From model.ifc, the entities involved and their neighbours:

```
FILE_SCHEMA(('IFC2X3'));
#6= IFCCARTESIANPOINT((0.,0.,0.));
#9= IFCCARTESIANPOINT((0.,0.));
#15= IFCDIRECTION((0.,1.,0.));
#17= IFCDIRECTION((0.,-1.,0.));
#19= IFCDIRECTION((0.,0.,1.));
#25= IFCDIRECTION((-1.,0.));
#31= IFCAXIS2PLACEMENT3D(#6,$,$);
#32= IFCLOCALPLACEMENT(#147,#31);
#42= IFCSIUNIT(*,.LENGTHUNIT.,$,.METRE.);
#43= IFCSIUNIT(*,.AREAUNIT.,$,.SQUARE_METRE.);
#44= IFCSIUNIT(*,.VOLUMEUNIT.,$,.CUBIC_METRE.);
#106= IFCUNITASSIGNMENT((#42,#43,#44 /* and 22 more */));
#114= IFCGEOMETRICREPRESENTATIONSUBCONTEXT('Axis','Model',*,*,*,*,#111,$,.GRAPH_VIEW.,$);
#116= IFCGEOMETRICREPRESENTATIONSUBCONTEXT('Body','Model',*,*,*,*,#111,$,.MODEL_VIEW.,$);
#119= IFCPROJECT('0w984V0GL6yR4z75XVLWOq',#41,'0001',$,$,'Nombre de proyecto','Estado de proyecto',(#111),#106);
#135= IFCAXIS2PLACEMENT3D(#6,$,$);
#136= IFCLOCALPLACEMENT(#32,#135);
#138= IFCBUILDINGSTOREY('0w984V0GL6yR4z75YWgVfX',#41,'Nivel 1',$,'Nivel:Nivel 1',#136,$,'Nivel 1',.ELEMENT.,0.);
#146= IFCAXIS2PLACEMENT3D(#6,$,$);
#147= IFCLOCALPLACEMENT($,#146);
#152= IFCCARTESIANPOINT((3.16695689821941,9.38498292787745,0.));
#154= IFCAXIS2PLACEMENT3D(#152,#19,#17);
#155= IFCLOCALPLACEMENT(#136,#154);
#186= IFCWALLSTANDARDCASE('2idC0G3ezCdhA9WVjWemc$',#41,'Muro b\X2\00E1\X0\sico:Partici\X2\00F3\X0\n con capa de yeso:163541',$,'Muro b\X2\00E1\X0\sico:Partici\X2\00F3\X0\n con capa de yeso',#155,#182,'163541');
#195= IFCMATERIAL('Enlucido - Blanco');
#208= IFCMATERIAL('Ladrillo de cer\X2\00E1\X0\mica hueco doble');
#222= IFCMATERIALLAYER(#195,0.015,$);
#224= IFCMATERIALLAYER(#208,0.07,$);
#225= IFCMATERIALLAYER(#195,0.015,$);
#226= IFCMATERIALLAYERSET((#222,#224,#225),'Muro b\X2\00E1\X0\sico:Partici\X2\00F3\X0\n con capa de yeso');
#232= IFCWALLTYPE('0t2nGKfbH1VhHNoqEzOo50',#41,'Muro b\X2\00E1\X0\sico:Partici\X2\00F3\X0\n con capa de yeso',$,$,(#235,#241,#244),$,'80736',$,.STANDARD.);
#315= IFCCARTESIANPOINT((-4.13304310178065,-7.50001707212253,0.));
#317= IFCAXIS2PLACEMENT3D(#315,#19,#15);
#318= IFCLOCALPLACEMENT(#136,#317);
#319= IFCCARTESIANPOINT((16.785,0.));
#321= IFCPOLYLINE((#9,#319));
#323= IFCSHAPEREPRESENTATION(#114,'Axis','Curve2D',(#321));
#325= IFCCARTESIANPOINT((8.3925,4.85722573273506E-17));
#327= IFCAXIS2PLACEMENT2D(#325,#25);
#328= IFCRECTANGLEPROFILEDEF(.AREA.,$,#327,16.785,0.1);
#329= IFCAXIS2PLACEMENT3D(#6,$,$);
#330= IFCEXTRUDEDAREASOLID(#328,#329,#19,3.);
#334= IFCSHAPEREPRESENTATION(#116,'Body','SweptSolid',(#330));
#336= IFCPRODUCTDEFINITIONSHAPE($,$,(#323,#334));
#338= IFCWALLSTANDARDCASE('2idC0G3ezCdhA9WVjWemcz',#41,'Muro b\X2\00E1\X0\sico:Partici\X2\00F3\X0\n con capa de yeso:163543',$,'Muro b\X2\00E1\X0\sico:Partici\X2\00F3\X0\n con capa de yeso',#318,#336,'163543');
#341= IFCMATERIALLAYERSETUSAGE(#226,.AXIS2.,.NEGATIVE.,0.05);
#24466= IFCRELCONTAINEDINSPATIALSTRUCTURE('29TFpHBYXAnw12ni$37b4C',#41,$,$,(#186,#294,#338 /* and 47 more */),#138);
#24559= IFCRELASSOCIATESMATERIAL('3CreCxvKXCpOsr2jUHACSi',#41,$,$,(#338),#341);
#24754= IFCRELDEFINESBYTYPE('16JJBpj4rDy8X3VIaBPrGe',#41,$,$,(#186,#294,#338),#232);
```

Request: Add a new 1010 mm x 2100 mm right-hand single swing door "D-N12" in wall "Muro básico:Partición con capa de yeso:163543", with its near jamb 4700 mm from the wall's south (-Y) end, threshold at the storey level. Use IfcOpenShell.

```python
import numpy as np
import ifcopenshell
import ifcopenshell.api.feature
import ifcopenshell.api.geometry
import ifcopenshell.api.root
import ifcopenshell.api.spatial
import ifcopenshell.api.type
import ifcopenshell.geom
import ifcopenshell.util.element
import ifcopenshell.util.placement
import ifcopenshell.util.representation
import ifcopenshell.util.shape
import ifcopenshell.util.unit

model = ifcopenshell.open("model.ifc")
unit_scale = ifcopenshell.util.unit.calculate_unit_scale(model)
settings = ifcopenshell.geom.settings()


def volume(element):
    """Net volume in cubic metres, openings subtracted."""
    shape = ifcopenshell.geom.create_shape(settings, element)
    return ifcopenshell.util.shape.get_volume(shape.geometry)


wall = model.by_id(338)
storey = ifcopenshell.util.element.get_container(wall, ifc_class="IfcBuildingStorey")
context = ifcopenshell.util.representation.get_context(model, "Model", "Body", "MODEL_VIEW")
before = volume(wall)

width, height, from_end, sill = 1.01, 2.1, 4.7, 0.0  # metres

# The wall runs along its own X axis, and the end named is its -X end.
wall_shape = ifcopenshell.geom.create_shape(settings, wall)
x, y, z = ifcopenshell.util.shape.get_vertices(wall_shape.geometry).T
start = x.min() + from_end
face, thickness = float(y.min()), float(y.max() - y.min())
wall_matrix = ifcopenshell.util.placement.get_local_placement(wall.ObjectPlacement)
level = ifcopenshell.util.placement.get_local_placement(storey.ObjectPlacement)[2, 3]


def in_wall(x, y):
    """Placement at x, y metres in the wall's axes, at sill height."""
    matrix = wall_matrix.copy()
    matrix[:, 3] = wall_matrix @ np.array([x / unit_scale, y / unit_scale, 0.0, 1.0])
    matrix[2, 3] = level + sill / unit_scale
    return matrix


# Opening: a box that overshoots both wall faces by 50 mm.
opening = ifcopenshell.api.root.create_entity(model, ifc_class="IfcOpeningElement")
box = ifcopenshell.api.geometry.add_wall_representation(
    model, context=context, length=width, height=height, thickness=thickness + 0.1
)
ifcopenshell.api.geometry.assign_representation(model, product=opening, representation=box)
ifcopenshell.api.geometry.edit_object_placement(model, product=opening, matrix=in_wall(start, face - 0.05), is_si=False)
ifcopenshell.api.feature.add_feature(model, feature=opening, element=wall)

door = ifcopenshell.api.root.create_entity(model, ifc_class="IfcDoor", name="D-N12")
door.OverallWidth, door.OverallHeight = width / unit_scale, height / unit_scale
body = ifcopenshell.api.geometry.add_door_representation(
    model,
    context=context,
    overall_width=door.OverallWidth,
    overall_height=door.OverallHeight,
    operation_type="SINGLE_SWING_RIGHT",
    lining_properties={"LiningDepth": thickness / unit_scale, "ThresholdDepth": thickness / unit_scale},
)
ifcopenshell.api.geometry.assign_representation(model, product=door, representation=body)
ifcopenshell.api.spatial.assign_container(model, products=[door], relating_structure=storey)
fills = ifcopenshell.api.feature.add_filling(model, opening=opening, element=door)
fills.OwnerHistory = door.OwnerHistory  # required in IFC2X3

# IFC2X3 keeps the operation on the door style.
style = ifcopenshell.api.root.create_entity(model, ifc_class="IfcDoorStyle", name="D-N12")
style.OperationType, style.ConstructionType = "SINGLE_SWING_RIGHT", "NOTDEFINED"
style.ParameterTakesPrecedence = style.Sizeable = False
ifcopenshell.api.type.assign_type(model, related_objects=[door], relating_type=style)

# The lining spans the wall, so the door starts at the wall face.
ifcopenshell.api.geometry.edit_object_placement(model, product=door, matrix=in_wall(start, face), is_si=False)

after = volume(wall)

print(f"wall volume {before:.3f} -> {after:.3f} m3")

model.write("model_v2.ifc")
```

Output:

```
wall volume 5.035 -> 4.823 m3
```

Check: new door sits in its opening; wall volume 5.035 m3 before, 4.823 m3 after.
